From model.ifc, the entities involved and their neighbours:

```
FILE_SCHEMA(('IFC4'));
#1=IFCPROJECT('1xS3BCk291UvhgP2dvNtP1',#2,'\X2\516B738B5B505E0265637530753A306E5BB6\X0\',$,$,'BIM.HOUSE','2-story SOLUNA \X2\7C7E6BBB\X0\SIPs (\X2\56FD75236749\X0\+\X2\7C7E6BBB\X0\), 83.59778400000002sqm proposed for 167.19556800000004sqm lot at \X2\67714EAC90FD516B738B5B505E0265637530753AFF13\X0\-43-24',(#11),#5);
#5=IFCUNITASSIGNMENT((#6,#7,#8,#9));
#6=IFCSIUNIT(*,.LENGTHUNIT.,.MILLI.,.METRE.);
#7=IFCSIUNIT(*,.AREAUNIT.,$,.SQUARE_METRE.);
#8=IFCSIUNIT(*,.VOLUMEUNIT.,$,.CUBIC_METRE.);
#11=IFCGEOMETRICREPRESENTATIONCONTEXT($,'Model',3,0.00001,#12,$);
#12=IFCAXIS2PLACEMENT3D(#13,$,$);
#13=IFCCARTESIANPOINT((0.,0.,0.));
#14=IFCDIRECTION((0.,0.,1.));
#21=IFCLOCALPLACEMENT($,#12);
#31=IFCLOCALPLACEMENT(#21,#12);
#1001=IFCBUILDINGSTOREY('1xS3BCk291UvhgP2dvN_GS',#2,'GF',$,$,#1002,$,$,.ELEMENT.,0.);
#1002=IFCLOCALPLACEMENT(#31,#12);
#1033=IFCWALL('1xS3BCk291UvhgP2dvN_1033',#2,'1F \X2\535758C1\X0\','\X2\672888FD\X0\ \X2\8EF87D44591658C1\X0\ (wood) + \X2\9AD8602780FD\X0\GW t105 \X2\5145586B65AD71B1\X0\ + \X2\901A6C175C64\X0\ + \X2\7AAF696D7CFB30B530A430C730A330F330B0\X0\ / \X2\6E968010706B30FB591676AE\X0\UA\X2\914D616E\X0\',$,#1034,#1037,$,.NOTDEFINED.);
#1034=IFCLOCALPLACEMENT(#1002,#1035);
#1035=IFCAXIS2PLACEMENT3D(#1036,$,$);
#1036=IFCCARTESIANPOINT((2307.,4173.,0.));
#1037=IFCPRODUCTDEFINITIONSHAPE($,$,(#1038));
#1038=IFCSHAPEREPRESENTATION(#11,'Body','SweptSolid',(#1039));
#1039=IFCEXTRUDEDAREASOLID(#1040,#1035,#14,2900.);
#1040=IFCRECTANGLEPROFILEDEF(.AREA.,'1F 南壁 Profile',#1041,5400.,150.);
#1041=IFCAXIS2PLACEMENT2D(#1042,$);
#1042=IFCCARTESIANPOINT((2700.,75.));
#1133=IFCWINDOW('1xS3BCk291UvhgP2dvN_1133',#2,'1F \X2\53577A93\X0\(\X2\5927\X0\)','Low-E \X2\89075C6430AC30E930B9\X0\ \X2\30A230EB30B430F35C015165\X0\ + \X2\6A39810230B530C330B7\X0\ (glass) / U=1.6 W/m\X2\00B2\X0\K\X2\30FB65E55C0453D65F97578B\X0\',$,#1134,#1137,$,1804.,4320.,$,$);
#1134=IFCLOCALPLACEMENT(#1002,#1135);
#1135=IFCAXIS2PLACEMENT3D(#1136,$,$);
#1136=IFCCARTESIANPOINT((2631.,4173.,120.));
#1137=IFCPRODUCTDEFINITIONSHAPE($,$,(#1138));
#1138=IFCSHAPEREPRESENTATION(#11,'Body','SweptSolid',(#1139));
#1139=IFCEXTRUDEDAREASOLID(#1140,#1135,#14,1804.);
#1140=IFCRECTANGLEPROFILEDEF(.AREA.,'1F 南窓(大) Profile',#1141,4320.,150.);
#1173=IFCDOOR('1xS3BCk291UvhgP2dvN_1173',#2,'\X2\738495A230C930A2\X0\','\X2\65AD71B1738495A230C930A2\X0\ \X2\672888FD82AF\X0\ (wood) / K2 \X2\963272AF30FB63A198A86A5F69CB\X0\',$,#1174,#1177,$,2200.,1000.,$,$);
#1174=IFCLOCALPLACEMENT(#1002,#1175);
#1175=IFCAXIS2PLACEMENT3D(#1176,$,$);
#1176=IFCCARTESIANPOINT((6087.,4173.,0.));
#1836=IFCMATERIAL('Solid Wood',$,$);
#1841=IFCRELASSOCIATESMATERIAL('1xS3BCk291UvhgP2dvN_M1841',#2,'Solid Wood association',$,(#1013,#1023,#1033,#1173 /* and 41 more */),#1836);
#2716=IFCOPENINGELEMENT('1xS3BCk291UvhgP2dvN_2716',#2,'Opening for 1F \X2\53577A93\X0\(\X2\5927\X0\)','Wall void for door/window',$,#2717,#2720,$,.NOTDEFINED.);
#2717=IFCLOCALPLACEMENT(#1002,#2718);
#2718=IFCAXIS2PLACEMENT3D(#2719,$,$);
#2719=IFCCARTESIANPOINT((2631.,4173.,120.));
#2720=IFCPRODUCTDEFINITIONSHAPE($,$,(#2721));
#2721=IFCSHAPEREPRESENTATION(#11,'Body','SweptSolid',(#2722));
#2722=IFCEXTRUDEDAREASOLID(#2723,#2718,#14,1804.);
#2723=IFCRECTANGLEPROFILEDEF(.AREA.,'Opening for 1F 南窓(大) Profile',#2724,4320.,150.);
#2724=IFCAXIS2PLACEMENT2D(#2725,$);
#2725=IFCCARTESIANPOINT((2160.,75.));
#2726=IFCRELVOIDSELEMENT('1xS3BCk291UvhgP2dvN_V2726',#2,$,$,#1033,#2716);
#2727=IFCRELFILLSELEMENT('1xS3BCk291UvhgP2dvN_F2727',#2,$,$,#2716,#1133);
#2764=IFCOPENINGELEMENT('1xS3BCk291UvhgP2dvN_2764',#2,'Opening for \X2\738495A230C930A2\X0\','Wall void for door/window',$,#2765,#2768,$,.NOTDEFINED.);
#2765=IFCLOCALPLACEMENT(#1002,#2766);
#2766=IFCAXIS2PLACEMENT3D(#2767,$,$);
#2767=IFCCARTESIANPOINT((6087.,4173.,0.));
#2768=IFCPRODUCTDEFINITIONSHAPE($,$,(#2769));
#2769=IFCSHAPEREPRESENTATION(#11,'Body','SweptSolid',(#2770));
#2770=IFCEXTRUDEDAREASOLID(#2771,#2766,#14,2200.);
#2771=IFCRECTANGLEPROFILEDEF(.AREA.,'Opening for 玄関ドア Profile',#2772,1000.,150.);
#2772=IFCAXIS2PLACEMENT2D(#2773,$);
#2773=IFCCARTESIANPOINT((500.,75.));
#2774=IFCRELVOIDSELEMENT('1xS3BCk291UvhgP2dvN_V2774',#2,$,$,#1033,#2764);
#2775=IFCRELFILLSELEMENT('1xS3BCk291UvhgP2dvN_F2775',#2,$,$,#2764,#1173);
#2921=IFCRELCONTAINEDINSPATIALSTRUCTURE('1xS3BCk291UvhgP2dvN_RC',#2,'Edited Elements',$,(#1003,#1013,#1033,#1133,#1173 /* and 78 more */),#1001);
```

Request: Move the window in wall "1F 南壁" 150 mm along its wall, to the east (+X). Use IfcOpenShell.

```python
import ifcopenshell
import ifcopenshell.api.geometry
import ifcopenshell.util.placement
import ifcopenshell.util.unit

model = ifcopenshell.open("model.ifc")
unit_scale = ifcopenshell.util.unit.calculate_unit_scale(model)

window = model.by_id(1133)
opening = window.FillsVoids[0].RelatingOpeningElement
wall = opening.VoidsElements[0].RelatingBuildingElement

wall_matrix = ifcopenshell.util.placement.get_local_placement(wall.ObjectPlacement)
shift = wall_matrix[:3, 0] * 0.15 / unit_scale
before = ifcopenshell.util.placement.get_local_placement(window.ObjectPlacement)[:3, 3].copy()

# The window is not placed relative to its opening, so move both.
for product in (opening, window):
    matrix = ifcopenshell.util.placement.get_local_placement(product.ObjectPlacement)
    matrix[:3, 3] += shift
    ifcopenshell.api.geometry.edit_object_placement(model, product=product, matrix=matrix, is_si=False)

after = ifcopenshell.util.placement.get_local_placement(window.ObjectPlacement)[:3, 3]
print("window moved by", (after - before).round(3) + 0.0)

model.write("model_v2.ifc")
```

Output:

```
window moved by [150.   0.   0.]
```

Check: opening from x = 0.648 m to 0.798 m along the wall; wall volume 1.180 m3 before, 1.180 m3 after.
